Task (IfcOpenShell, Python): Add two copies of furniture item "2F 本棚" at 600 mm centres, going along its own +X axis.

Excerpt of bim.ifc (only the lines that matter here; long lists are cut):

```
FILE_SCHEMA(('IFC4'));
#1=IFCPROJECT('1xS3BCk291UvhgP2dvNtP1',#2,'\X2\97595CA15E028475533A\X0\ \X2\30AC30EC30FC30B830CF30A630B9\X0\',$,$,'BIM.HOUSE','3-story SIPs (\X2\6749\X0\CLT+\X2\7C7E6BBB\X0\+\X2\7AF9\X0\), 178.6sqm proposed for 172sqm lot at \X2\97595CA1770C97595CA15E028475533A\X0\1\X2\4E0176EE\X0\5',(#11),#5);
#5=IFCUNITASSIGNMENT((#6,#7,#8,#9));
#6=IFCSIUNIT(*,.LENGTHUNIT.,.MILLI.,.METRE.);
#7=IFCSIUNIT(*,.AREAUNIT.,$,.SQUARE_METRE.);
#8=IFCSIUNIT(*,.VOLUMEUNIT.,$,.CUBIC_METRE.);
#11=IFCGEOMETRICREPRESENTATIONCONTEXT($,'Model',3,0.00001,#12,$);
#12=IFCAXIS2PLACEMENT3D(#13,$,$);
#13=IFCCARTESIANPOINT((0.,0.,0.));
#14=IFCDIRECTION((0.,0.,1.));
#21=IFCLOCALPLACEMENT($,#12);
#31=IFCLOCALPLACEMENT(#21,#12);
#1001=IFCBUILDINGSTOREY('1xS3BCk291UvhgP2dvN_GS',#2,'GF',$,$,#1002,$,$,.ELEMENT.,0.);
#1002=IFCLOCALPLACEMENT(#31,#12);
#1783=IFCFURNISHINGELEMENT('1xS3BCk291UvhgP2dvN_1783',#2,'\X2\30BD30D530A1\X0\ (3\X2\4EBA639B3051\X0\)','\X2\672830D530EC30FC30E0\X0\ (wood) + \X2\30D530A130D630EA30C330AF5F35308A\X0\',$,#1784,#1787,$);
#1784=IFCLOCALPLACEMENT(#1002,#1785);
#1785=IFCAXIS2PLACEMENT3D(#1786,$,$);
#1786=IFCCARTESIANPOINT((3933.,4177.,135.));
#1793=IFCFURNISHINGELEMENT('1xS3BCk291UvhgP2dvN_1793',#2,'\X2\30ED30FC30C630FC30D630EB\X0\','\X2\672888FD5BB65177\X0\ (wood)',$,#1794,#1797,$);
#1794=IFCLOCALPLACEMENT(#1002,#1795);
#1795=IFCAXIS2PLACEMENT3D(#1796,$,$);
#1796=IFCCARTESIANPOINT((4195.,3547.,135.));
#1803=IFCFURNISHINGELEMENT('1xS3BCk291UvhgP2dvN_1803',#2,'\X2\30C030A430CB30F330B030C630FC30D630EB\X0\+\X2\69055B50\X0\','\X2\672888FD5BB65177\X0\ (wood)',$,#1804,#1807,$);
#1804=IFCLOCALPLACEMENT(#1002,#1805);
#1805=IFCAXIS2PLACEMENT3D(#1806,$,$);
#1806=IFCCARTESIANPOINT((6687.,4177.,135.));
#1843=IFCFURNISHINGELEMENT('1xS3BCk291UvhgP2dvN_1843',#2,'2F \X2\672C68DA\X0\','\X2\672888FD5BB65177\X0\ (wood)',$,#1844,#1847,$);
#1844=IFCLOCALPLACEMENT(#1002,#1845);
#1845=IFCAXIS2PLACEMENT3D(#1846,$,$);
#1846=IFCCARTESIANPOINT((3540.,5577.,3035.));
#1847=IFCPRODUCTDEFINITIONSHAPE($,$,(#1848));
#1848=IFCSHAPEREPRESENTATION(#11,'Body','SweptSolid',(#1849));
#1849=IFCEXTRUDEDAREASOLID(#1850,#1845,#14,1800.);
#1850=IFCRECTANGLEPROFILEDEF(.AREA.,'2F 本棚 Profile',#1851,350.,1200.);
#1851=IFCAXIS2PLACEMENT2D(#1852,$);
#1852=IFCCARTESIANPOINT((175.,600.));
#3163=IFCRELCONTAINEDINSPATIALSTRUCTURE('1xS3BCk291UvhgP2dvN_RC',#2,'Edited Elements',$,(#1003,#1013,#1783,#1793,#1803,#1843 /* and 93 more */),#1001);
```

```python
import ifcopenshell
import ifcopenshell.api.geometry
import ifcopenshell.api.root
import ifcopenshell.util.element
import ifcopenshell.util.placement

model = ifcopenshell.open("bim.ifc")


def reuse_history(source, copy):
    """copy_class also copies each property set's owner history, people and application; keep the originals."""
    for rel in copy.IsDefinedBy:
        if rel.is_a("IfcRelDefinesByProperties") and (history := rel.RelatingPropertyDefinition.OwnerHistory):
            rel.RelatingPropertyDefinition.OwnerHistory = source.OwnerHistory
            ifcopenshell.util.element.remove_deep2(model, history)


source = model.by_guid("1xS3BCk291UvhgP2dvN_1843")
base = ifcopenshell.util.placement.get_local_placement(source.ObjectPlacement)
step = base[:3, 0] * 600.0

for i in range(1, 3):
    copy = ifcopenshell.api.root.copy_class(model, product=source)
    copy.Representation = ifcopenshell.util.element.copy_deep(
        model, source.Representation, exclude=["IfcGeometricRepresentationContext", "IfcRepresentationMap"]
    )
    reuse_history(source, copy)
    matrix = base.copy()
    matrix[:3, 3] += i * step
    print("added at", matrix[:3, 3].round(3) + 0.0)
    ifcopenshell.api.geometry.edit_object_placement(model, product=copy, matrix=matrix, is_si=False)

model.write("bim_v2.ifc")
```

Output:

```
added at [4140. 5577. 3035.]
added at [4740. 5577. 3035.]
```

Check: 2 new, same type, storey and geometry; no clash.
